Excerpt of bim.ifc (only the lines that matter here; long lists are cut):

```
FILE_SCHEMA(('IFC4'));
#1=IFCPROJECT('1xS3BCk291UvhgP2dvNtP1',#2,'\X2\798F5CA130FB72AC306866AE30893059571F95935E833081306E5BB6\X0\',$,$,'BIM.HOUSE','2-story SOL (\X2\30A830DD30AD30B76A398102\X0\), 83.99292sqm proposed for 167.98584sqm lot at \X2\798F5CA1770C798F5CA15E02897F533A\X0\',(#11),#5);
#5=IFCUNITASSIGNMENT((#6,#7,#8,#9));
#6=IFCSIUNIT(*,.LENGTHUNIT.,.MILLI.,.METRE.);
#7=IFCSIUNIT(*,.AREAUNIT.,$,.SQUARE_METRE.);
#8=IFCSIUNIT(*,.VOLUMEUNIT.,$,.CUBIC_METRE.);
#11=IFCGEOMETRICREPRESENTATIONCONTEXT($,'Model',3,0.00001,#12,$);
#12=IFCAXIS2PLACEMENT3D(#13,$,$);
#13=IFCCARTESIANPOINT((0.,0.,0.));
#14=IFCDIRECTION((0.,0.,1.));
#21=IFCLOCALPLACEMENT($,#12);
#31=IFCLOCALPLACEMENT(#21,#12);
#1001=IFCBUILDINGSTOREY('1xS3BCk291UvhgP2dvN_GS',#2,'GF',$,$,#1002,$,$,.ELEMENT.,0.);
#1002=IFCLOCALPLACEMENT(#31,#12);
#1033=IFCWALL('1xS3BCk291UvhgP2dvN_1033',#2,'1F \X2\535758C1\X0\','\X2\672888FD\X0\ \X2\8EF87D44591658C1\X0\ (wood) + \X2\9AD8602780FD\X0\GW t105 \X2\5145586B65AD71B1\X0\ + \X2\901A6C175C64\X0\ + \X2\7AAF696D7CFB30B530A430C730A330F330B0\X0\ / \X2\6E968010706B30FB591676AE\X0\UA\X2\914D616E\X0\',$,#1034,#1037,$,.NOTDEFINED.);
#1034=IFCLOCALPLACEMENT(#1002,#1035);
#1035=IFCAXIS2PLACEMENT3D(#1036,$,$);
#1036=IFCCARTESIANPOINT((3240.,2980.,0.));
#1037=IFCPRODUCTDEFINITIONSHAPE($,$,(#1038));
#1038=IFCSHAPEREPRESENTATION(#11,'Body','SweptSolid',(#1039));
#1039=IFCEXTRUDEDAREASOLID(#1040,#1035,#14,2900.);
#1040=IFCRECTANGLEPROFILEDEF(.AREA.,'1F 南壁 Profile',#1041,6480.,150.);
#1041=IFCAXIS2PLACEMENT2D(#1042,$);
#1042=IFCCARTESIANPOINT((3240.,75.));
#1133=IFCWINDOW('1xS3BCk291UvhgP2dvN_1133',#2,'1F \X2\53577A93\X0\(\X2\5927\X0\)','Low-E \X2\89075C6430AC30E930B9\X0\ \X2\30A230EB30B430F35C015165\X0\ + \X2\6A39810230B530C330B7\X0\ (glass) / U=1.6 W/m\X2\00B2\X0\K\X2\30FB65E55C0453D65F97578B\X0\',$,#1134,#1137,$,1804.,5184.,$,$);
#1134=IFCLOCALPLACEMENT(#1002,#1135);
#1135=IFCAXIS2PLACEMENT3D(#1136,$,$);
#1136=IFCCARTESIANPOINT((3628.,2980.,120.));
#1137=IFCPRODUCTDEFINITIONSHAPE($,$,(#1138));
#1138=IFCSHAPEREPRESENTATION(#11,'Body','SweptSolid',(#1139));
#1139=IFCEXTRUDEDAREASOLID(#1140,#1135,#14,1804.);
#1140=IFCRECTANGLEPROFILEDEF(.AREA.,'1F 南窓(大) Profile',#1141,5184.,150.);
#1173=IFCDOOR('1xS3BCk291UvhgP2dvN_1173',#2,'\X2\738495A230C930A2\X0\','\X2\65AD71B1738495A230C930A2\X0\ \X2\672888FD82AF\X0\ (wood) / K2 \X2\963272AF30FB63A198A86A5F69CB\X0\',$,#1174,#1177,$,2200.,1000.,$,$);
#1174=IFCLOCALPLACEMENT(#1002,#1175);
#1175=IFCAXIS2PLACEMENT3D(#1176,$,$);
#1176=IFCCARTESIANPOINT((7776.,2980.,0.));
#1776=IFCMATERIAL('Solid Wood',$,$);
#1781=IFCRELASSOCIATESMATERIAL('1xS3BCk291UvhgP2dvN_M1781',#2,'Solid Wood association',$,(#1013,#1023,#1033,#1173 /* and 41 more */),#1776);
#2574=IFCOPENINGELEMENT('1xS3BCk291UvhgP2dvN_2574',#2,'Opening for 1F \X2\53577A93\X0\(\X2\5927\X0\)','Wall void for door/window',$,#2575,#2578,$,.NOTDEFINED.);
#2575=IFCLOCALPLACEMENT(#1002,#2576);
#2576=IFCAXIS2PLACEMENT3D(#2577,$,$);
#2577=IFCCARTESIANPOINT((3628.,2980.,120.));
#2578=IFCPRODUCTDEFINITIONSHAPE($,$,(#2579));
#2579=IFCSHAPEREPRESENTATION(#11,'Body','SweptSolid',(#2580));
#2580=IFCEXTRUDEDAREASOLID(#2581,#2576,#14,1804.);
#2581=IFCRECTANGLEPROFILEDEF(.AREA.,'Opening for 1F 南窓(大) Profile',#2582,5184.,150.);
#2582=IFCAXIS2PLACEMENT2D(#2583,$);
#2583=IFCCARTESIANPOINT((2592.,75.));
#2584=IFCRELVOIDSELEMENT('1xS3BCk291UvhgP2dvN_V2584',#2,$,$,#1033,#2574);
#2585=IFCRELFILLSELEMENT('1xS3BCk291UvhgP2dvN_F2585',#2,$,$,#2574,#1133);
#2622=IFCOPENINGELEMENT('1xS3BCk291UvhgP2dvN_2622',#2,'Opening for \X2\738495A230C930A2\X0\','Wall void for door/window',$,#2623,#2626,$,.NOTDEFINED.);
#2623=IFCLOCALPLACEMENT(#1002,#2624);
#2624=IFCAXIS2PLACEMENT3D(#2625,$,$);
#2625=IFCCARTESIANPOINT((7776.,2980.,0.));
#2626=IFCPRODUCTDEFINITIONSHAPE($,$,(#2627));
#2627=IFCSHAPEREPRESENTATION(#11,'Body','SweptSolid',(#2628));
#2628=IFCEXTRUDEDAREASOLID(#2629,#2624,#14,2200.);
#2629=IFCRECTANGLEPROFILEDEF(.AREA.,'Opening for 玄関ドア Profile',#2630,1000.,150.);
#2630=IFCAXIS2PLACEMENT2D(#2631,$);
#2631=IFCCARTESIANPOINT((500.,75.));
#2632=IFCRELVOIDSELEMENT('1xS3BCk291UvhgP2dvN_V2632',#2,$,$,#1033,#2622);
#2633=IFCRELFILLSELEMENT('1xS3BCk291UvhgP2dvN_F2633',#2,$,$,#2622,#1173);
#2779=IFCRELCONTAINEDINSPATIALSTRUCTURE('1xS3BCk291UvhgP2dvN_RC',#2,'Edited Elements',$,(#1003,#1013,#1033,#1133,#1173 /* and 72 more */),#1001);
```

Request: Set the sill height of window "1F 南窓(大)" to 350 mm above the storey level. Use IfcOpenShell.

```python
import numpy as np
import ifcopenshell
import ifcopenshell.api.geometry
import ifcopenshell.geom
import ifcopenshell.util.element
import ifcopenshell.util.placement
import ifcopenshell.util.shape
import ifcopenshell.util.unit

model = ifcopenshell.open("bim.ifc")
unit_scale = ifcopenshell.util.unit.calculate_unit_scale(model)

window = model.by_id(1133)
opening = window.FillsVoids[0].RelatingOpeningElement
storey = ifcopenshell.util.element.get_container(window, ifc_class="IfcBuildingStorey")
level = ifcopenshell.util.placement.get_local_placement(storey.ObjectPlacement)[2, 3]

# The opening's origin need not be at the sill, so measure its lowest point.
shape = ifcopenshell.geom.create_shape(ifcopenshell.geom.settings(), opening)
bottom = ifcopenshell.util.shape.get_shape_bottom_elevation(shape, shape.geometry) / unit_scale
dz = level + 350.0 - bottom

shift = np.array([0.0, 0.0, dz])
# The window is not placed relative to its opening, so move both.
for product in (opening, window):
    matrix = ifcopenshell.util.placement.get_local_placement(product.ObjectPlacement)
    matrix[:3, 3] += shift
    ifcopenshell.api.geometry.edit_object_placement(model, product=product, matrix=matrix, is_si=False)

print(f"moved by {dz * unit_scale:+.3f} m")

model.write("bim_updated.ifc")
```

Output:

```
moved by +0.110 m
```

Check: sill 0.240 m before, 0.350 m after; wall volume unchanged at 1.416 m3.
